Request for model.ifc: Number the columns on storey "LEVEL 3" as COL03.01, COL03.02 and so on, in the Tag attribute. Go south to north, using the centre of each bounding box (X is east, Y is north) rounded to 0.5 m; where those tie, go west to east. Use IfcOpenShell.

First a look at what the model holds.

```python
import ifcopenshell
import ifcopenshell.util.element
import ifcopenshell.util.placement

model = ifcopenshell.open("model.ifc")
print(model.schema)
storey = next(s for s in model.by_type("IfcBuildingStorey") if s.Name == "LEVEL 3")
columns = [e for e in ifcopenshell.util.element.get_decomposition(storey) if e.is_a("IfcColumn")]
for e in sorted(columns, key=lambda e: e.id()):
    origin = ifcopenshell.util.placement.get_local_placement(e.ObjectPlacement)[:3, 3]
    print(e.id(), e.Tag, e.Name, origin.round(2) + 0.0, sep=" | ")
```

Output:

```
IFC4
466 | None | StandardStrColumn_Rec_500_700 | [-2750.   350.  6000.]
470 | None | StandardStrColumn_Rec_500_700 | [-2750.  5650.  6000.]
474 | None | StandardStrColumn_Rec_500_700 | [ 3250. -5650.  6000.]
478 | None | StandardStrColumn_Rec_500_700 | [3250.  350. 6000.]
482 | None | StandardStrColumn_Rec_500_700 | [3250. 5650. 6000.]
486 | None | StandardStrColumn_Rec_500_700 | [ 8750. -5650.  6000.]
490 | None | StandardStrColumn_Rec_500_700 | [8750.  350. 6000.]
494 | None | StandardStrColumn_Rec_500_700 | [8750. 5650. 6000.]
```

```python
import ifcopenshell
import ifcopenshell.geom
import ifcopenshell.util.element
import ifcopenshell.util.shape

model = ifcopenshell.open("model.ifc")
settings = ifcopenshell.geom.settings()
settings.set("use-world-coords", True)


def centre(element):
    shape = ifcopenshell.geom.create_shape(settings, element)
    return ifcopenshell.util.shape.get_bbox_centroid(shape.geometry)


storey = next(s for s in model.by_type("IfcBuildingStorey") if s.Name == "LEVEL 3")
columns = [e for e in ifcopenshell.util.element.get_decomposition(storey) if e.is_a("IfcColumn")]

# Insertion points can sit at a corner or the storey origin, so sort by the geometry (in metres).
centres = {e: centre(e) for e in columns}
columns.sort(key=lambda e: (round(centres[e][1] / 0.5), centres[e][0]))

for i, e in enumerate(columns, start=1):
    number = f"COL03.{i:02d}"
    e.Tag = number
    print(e.id(), number)

model.write("model-out.ifc")
```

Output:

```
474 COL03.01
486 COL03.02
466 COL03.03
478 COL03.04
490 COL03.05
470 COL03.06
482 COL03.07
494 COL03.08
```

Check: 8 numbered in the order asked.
